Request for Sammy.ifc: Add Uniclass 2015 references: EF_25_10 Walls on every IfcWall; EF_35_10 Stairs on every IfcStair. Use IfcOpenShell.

First a look at what the model holds.

```python
import ifcopenshell

model = ifcopenshell.open("Sammy.ifc")
print(model.schema)
print("classifications:", [c.Name for c in model.by_type("IfcClassification")])
for ifc_class in ("IfcDoor", "IfcRoof", "IfcStair", "IfcWall", "IfcWindow"):
    print(ifc_class, len(model.by_type(ifc_class)))
```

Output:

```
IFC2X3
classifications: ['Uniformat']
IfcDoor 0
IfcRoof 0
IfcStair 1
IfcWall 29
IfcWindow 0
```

```python
import ifcopenshell
import ifcopenshell.api.classification

model = ifcopenshell.open("Sammy.ifc")

# IFC2X3 requires Source and Edition and has no link from the project to the system.
system = model.create_entity("IfcClassification", Source="NBS", Edition="2015", Name="Uniclass 2015")

codes = {
    "IfcWall": ("EF_25_10", "Walls"),
    "IfcStair": ("EF_35_10", "Stairs"),
}
for ifc_class, (code, name) in codes.items():
    products = model.by_type(ifc_class)
    ifcopenshell.api.classification.add_reference(
        model, products=products, classification=system, identification=code, name=name
    )
    print(code, len(products))

model.write("Sammy_edited.ifc")
```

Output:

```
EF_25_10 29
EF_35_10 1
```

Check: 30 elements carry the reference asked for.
